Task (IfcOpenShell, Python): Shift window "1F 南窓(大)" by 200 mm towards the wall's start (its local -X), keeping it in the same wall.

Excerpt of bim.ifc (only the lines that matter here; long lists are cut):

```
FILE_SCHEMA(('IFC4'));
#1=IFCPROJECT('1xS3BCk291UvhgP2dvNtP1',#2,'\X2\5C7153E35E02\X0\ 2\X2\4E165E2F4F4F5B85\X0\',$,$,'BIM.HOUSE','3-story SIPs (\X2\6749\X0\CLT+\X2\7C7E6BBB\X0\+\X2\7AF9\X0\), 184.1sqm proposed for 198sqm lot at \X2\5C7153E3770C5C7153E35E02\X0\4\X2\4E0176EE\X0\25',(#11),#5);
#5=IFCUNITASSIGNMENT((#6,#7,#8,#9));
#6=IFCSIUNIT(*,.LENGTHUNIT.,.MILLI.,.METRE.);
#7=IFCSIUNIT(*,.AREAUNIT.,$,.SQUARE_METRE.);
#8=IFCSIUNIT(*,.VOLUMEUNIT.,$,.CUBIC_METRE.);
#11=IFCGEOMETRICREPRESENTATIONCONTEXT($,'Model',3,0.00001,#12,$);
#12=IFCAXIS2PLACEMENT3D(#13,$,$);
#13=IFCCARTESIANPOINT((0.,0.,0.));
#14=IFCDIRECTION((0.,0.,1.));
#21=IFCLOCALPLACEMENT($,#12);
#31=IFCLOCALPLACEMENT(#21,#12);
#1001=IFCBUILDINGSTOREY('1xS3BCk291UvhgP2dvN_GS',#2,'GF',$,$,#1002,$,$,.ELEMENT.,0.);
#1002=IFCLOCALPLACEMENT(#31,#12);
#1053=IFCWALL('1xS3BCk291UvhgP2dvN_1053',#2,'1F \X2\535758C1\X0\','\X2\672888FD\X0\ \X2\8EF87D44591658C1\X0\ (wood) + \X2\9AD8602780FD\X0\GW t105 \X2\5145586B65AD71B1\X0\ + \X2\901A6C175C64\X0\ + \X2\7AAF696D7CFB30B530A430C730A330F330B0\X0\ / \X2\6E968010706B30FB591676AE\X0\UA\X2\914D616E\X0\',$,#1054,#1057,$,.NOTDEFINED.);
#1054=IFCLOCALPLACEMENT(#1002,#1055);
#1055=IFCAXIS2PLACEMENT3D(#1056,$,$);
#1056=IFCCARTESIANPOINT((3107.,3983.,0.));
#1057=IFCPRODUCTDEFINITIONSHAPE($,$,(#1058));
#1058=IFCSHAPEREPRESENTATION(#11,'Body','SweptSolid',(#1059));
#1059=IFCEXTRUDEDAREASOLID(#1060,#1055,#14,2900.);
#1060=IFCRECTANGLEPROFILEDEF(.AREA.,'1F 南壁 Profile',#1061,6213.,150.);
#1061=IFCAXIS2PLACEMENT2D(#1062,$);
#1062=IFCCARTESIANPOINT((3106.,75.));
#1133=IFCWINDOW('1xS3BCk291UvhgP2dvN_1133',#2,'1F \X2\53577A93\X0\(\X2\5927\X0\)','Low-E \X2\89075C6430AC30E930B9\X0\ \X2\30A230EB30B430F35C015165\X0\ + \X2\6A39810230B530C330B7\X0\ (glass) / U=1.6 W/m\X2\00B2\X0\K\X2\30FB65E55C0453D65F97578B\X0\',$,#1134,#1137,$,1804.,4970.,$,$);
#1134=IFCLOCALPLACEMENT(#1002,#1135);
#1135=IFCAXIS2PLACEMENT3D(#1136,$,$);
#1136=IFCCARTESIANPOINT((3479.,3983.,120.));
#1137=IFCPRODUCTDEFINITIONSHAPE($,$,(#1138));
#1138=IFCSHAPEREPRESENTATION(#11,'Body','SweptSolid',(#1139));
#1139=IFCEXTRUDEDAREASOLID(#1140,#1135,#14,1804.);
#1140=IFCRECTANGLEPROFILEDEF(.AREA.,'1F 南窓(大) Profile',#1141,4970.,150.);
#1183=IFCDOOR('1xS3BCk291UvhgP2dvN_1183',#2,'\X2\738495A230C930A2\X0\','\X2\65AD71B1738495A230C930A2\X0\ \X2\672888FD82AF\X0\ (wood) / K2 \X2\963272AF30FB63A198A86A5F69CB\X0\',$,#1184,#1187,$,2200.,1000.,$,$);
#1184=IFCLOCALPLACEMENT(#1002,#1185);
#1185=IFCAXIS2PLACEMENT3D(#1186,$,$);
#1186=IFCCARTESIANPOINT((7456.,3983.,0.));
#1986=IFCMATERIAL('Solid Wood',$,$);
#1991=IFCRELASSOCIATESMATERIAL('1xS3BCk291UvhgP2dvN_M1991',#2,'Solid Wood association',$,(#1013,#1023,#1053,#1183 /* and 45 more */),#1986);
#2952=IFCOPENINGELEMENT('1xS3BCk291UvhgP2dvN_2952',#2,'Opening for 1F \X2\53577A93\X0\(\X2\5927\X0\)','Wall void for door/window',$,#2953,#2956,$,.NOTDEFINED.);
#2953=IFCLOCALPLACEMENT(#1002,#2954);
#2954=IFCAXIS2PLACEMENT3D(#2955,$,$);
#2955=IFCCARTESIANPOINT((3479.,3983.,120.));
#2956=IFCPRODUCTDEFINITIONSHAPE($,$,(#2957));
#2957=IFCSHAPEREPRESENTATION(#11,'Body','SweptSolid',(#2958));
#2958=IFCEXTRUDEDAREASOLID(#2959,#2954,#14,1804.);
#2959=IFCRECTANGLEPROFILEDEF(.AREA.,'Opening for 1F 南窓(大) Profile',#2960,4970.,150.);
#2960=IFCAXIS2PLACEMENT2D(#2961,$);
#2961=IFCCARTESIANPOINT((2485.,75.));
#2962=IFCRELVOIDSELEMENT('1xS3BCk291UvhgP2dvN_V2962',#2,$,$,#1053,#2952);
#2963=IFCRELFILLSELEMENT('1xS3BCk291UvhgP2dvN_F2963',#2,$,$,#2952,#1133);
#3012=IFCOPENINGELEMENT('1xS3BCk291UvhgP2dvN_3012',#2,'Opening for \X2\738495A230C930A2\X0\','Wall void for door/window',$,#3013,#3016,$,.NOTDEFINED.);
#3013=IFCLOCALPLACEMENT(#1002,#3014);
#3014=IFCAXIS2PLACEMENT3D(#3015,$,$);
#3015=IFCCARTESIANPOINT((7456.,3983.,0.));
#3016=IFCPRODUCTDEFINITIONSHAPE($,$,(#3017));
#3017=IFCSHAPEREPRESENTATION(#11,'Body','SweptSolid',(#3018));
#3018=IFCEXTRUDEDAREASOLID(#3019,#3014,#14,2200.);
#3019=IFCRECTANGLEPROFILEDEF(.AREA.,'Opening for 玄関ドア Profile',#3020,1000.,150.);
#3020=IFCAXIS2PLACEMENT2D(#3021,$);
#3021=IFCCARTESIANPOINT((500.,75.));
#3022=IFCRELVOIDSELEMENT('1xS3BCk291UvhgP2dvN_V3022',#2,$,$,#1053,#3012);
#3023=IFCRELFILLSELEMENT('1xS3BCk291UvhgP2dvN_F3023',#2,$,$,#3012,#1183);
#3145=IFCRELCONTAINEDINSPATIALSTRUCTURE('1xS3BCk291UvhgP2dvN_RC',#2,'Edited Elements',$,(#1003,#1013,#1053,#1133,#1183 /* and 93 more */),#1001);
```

```python
import ifcopenshell
import ifcopenshell.api.geometry
import ifcopenshell.util.placement
import ifcopenshell.util.unit

model = ifcopenshell.open("bim.ifc")
unit_scale = ifcopenshell.util.unit.calculate_unit_scale(model)

window = model.by_id(1133)
opening = window.FillsVoids[0].RelatingOpeningElement
wall = opening.VoidsElements[0].RelatingBuildingElement

wall_matrix = ifcopenshell.util.placement.get_local_placement(wall.ObjectPlacement)
shift = wall_matrix[:3, 0] * -0.2 / unit_scale
before = ifcopenshell.util.placement.get_local_placement(window.ObjectPlacement)[:3, 3].copy()

# The window is not placed relative to its opening, so move both.
for product in (opening, window):
    matrix = ifcopenshell.util.placement.get_local_placement(product.ObjectPlacement)
    matrix[:3, 3] += shift
    ifcopenshell.api.geometry.edit_object_placement(model, product=product, matrix=matrix, is_si=False)

after = ifcopenshell.util.placement.get_local_placement(window.ObjectPlacement)[:3, 3]
print("window moved by", (after - before).round(3) + 0.0)

model.write("bim_v2.ifc")
```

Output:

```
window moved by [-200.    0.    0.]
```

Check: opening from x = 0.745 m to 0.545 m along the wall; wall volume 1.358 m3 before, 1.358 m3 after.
